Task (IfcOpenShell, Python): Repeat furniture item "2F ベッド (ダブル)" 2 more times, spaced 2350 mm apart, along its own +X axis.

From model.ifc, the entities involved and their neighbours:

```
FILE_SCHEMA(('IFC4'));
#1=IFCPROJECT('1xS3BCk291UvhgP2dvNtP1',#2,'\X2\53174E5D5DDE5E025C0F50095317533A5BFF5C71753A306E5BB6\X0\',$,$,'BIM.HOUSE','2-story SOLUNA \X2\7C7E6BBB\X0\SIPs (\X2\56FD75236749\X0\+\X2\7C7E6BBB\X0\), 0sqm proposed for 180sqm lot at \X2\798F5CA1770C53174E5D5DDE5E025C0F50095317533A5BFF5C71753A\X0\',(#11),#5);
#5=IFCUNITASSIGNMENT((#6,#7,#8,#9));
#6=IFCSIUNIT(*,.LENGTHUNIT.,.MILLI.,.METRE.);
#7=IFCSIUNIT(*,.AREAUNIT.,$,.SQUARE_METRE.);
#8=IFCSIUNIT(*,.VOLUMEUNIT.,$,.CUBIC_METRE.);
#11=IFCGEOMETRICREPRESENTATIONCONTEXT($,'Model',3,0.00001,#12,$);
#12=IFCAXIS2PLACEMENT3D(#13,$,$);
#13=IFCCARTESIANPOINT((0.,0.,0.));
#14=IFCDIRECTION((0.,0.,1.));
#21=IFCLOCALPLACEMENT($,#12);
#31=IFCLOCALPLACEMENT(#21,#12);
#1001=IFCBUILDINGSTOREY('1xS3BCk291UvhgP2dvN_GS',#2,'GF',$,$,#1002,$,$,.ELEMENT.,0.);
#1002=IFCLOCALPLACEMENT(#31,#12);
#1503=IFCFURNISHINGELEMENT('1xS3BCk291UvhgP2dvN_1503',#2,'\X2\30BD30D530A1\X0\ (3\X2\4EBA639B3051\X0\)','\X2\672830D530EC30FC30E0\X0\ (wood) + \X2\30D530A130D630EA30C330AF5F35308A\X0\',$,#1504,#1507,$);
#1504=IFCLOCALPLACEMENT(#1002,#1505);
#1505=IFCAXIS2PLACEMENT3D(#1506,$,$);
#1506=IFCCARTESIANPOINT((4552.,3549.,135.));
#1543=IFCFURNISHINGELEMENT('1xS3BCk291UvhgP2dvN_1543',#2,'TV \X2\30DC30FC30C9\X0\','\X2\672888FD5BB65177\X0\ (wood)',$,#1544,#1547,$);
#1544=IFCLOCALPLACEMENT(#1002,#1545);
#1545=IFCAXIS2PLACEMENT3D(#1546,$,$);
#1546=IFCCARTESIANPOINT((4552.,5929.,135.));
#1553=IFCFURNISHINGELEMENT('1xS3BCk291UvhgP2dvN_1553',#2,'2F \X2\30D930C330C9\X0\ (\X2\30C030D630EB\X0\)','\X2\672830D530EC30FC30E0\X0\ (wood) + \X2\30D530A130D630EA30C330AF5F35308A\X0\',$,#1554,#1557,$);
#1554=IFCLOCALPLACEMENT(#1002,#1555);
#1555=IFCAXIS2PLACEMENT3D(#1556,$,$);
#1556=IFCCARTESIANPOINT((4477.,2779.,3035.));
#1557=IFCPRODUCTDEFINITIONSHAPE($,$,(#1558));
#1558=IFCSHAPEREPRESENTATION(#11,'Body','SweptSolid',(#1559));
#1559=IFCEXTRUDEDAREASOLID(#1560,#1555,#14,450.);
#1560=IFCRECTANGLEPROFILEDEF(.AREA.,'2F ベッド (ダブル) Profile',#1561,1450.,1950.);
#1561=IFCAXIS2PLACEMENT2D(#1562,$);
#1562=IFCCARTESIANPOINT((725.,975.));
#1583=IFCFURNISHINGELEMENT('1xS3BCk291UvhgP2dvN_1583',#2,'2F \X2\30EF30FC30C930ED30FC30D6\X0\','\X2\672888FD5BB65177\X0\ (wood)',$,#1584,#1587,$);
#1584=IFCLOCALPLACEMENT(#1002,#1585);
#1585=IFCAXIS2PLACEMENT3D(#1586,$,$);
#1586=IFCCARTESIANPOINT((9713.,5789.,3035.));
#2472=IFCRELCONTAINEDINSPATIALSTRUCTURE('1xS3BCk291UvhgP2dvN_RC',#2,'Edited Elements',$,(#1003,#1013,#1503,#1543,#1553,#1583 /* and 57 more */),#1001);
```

```python
import ifcopenshell
import ifcopenshell.api.geometry
import ifcopenshell.api.root
import ifcopenshell.util.element
import ifcopenshell.util.placement
import ifcopenshell.util.unit

model = ifcopenshell.open("model.ifc")
unit_scale = ifcopenshell.util.unit.calculate_unit_scale(model)


def reuse_history(source, copy):
    """copy_class also copies each property set's owner history, people and application; keep the originals."""
    for rel in copy.IsDefinedBy:
        if rel.is_a("IfcRelDefinesByProperties") and (history := rel.RelatingPropertyDefinition.OwnerHistory):
            rel.RelatingPropertyDefinition.OwnerHistory = source.OwnerHistory
            ifcopenshell.util.element.remove_deep2(model, history)


source = model.by_guid("1xS3BCk291UvhgP2dvN_1553")
base = ifcopenshell.util.placement.get_local_placement(source.ObjectPlacement)
step = base[:3, 0] * 2.35 / unit_scale

for i in range(1, 3):
    copy = ifcopenshell.api.root.copy_class(model, product=source)
    copy.Representation = ifcopenshell.util.element.copy_deep(
        model, source.Representation, exclude=["IfcGeometricRepresentationContext", "IfcRepresentationMap"]
    )
    reuse_history(source, copy)
    matrix = base.copy()
    matrix[:3, 3] += i * step
    print("added at", matrix[:3, 3].round(3) + 0.0)
    ifcopenshell.api.geometry.edit_object_placement(model, product=copy, matrix=matrix, is_si=False)

model.write("model-out.ifc")
```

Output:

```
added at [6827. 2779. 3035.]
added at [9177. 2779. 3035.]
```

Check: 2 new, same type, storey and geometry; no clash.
